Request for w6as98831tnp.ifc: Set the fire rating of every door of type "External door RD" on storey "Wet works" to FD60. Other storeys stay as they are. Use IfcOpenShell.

First a look at what the model holds.

```python
import ifcopenshell
import ifcopenshell.util.element

model = ifcopenshell.open("w6as98831tnp.ifc")
print(model.schema)
storey = next(s for s in model.by_type("IfcBuildingStorey") if s.Name == "Wet works")
doors = [e for e in ifcopenshell.util.element.get_decomposition(storey) if e.is_a("IfcDoor")]
seen = {}
for e in doors:
    element_type = ifcopenshell.util.element.get_type(e)
    key = (element_type.Name if element_type != e and element_type else None, ifcopenshell.util.element.get_pset(e, "Pset_DoorCommon", "FireRating"))
    seen[key] = seen.get(key, 0) + 1
for (name, value), count in sorted(seen.items(), key=str):
    print(count, "x", name, "|", value)
```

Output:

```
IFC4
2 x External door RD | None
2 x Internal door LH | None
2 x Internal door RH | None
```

```python
import ifcopenshell
import ifcopenshell.api.pset
import ifcopenshell.util.element

model = ifcopenshell.open("w6as98831tnp.ifc")

storey = next(s for s in model.by_type("IfcBuildingStorey") if s.Name == "Wet works")
doors = [e for e in ifcopenshell.util.element.get_decomposition(storey) if e.is_a("IfcDoor")]

count = 0
for e in doors:
    element_type = ifcopenshell.util.element.get_type(e)
    if element_type in (None, e) or element_type.Name != "External door RD":
        continue
    # add_pset returns the element's existing set when there is one.
    pset = ifcopenshell.api.pset.add_pset(model, product=e, name="Pset_DoorCommon")
    ifcopenshell.api.pset.edit_pset(model, pset=pset, properties={"FireRating": "FD60"})
    count += 1

print(count, "doors updated")

model.write("w6as98831tnp_rev.ifc")
```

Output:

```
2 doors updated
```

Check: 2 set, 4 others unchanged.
